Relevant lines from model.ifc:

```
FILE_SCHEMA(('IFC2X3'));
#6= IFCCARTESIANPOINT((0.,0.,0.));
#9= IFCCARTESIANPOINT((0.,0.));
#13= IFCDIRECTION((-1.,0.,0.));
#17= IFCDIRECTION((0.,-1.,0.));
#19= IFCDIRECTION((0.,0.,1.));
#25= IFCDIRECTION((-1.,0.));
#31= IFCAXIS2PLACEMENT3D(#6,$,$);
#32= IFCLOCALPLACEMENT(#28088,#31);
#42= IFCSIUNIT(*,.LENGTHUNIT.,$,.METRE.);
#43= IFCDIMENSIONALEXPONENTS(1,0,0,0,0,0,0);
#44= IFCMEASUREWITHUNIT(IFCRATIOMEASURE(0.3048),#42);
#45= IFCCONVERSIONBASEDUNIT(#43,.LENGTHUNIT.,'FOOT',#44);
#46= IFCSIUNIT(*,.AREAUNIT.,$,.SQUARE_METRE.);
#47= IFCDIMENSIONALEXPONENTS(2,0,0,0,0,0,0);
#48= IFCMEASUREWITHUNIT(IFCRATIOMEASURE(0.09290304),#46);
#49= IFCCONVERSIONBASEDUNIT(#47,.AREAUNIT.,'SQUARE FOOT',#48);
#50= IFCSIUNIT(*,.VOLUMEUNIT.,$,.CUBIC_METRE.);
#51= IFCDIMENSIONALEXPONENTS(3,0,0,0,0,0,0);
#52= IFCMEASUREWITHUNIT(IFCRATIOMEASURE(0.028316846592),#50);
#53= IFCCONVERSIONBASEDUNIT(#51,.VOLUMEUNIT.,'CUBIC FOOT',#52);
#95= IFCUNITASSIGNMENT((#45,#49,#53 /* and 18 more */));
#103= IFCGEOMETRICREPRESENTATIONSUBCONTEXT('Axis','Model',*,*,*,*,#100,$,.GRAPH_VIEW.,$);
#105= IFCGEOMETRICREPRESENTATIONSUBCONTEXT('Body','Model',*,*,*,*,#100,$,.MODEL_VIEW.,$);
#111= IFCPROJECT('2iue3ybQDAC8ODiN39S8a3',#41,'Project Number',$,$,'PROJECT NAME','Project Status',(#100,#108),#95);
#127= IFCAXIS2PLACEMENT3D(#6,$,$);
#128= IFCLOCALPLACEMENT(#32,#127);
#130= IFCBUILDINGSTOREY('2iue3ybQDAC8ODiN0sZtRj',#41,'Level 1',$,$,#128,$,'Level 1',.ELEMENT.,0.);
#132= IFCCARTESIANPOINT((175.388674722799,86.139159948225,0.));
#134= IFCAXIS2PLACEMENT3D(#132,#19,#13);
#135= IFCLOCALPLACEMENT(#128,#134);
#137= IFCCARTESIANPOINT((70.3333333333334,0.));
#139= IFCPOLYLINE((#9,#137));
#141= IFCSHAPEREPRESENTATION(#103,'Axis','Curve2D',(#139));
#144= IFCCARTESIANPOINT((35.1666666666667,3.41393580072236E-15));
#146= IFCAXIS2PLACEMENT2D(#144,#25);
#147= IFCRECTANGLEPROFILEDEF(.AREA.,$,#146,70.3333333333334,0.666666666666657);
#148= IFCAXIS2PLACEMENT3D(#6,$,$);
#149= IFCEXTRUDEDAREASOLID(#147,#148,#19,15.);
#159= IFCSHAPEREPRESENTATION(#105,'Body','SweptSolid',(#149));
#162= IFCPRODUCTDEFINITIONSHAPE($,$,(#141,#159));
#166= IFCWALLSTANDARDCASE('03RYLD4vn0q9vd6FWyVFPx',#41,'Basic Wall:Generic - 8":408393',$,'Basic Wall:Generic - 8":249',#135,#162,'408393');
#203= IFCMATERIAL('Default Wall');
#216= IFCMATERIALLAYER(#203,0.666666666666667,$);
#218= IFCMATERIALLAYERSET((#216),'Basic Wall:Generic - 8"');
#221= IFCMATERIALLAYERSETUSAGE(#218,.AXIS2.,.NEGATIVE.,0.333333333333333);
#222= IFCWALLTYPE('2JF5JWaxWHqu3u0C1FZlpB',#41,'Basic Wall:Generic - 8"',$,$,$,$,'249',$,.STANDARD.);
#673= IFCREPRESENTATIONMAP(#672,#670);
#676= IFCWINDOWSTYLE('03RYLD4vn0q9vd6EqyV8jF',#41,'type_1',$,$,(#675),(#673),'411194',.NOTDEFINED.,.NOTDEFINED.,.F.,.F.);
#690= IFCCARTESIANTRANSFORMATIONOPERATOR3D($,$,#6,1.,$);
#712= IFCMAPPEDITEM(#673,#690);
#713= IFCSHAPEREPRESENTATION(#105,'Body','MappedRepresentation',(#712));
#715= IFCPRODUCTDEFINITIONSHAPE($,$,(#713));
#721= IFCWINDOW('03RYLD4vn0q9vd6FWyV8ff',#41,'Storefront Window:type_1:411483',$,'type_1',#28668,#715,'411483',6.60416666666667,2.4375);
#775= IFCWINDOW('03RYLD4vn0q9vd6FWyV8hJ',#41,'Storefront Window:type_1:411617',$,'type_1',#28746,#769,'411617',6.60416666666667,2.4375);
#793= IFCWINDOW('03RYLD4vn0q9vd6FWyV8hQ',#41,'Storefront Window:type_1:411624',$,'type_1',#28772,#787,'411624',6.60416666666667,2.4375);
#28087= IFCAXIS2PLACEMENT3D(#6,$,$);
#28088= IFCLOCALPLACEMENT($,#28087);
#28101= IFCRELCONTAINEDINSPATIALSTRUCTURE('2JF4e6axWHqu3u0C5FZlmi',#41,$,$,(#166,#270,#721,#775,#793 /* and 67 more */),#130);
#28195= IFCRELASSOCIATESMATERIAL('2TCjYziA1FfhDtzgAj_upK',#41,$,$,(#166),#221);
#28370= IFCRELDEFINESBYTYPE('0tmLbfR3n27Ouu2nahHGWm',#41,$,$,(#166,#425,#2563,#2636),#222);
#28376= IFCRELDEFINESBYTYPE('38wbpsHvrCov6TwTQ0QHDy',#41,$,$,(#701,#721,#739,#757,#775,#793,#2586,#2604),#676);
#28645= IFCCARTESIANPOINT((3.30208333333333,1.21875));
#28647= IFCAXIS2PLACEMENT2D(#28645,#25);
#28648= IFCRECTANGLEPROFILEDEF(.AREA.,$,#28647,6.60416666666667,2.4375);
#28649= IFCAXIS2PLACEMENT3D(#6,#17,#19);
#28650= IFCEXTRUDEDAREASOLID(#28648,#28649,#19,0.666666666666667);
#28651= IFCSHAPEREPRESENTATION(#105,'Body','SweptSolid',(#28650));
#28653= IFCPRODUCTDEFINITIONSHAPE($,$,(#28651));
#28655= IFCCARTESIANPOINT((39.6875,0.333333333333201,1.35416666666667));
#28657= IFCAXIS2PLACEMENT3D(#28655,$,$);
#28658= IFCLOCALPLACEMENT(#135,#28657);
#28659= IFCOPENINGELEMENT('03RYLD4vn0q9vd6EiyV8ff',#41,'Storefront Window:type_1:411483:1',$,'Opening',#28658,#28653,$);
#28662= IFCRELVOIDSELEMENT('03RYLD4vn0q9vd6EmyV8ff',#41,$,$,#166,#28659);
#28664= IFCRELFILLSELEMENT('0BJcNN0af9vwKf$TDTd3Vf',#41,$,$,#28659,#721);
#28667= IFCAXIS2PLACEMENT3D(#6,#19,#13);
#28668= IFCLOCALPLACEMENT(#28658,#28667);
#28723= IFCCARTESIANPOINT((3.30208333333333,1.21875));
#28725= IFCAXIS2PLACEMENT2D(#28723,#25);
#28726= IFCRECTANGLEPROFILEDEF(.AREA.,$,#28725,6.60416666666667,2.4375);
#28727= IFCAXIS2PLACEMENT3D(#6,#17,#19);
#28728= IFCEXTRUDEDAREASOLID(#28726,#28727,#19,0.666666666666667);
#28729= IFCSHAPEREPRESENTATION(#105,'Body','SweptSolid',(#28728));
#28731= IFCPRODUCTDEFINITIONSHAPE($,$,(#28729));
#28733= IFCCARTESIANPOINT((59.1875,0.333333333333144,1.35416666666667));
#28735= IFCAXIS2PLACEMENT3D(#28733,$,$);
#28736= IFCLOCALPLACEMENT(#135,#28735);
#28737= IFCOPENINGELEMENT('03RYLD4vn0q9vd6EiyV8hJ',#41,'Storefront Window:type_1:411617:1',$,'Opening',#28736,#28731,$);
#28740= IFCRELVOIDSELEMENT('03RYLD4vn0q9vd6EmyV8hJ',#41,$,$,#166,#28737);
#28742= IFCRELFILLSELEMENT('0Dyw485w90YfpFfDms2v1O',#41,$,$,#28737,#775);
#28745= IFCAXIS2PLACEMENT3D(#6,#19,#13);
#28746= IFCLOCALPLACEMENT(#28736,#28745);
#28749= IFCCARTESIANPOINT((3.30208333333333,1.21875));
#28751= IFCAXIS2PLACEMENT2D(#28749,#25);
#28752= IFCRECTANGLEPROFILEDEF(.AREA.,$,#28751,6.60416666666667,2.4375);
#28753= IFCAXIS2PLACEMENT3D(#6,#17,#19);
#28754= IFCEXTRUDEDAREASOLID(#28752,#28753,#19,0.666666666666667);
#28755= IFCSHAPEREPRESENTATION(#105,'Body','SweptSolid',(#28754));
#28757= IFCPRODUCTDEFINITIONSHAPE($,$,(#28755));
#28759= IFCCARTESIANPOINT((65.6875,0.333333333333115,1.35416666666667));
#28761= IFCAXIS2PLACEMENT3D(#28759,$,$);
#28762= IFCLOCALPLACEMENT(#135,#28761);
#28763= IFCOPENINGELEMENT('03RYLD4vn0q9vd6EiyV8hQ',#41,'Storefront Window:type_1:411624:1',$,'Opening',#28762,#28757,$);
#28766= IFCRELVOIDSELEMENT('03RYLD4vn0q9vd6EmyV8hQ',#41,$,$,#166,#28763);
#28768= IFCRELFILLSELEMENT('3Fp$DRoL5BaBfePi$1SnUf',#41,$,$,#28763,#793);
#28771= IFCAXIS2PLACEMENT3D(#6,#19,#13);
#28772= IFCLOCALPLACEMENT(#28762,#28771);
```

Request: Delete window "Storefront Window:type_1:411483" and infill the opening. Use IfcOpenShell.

```python
import ifcopenshell
import ifcopenshell.api.feature
import ifcopenshell.api.root
import ifcopenshell.geom
import ifcopenshell.util.shape

model = ifcopenshell.open("model.ifc")
settings = ifcopenshell.geom.settings()


def volume(element):
    """Net volume in cubic metres, openings subtracted."""
    shape = ifcopenshell.geom.create_shape(settings, element)
    return ifcopenshell.util.shape.get_volume(shape.geometry)


window = model.by_guid("03RYLD4vn0q9vd6FWyV8ff")
opening = window.FillsVoids[0].RelatingOpeningElement
wall = opening.VoidsElements[0].RelatingBuildingElement
before = volume(wall)

ifcopenshell.api.root.remove_product(model, product=window)
ifcopenshell.api.feature.remove_feature(model, feature=opening)

after = volume(wall)

print(f"wall volume {before:.3f} -> {after:.3f} m3")

model.write("model_edited.ifc")
```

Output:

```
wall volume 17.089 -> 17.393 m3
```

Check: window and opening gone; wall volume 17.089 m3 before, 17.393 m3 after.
